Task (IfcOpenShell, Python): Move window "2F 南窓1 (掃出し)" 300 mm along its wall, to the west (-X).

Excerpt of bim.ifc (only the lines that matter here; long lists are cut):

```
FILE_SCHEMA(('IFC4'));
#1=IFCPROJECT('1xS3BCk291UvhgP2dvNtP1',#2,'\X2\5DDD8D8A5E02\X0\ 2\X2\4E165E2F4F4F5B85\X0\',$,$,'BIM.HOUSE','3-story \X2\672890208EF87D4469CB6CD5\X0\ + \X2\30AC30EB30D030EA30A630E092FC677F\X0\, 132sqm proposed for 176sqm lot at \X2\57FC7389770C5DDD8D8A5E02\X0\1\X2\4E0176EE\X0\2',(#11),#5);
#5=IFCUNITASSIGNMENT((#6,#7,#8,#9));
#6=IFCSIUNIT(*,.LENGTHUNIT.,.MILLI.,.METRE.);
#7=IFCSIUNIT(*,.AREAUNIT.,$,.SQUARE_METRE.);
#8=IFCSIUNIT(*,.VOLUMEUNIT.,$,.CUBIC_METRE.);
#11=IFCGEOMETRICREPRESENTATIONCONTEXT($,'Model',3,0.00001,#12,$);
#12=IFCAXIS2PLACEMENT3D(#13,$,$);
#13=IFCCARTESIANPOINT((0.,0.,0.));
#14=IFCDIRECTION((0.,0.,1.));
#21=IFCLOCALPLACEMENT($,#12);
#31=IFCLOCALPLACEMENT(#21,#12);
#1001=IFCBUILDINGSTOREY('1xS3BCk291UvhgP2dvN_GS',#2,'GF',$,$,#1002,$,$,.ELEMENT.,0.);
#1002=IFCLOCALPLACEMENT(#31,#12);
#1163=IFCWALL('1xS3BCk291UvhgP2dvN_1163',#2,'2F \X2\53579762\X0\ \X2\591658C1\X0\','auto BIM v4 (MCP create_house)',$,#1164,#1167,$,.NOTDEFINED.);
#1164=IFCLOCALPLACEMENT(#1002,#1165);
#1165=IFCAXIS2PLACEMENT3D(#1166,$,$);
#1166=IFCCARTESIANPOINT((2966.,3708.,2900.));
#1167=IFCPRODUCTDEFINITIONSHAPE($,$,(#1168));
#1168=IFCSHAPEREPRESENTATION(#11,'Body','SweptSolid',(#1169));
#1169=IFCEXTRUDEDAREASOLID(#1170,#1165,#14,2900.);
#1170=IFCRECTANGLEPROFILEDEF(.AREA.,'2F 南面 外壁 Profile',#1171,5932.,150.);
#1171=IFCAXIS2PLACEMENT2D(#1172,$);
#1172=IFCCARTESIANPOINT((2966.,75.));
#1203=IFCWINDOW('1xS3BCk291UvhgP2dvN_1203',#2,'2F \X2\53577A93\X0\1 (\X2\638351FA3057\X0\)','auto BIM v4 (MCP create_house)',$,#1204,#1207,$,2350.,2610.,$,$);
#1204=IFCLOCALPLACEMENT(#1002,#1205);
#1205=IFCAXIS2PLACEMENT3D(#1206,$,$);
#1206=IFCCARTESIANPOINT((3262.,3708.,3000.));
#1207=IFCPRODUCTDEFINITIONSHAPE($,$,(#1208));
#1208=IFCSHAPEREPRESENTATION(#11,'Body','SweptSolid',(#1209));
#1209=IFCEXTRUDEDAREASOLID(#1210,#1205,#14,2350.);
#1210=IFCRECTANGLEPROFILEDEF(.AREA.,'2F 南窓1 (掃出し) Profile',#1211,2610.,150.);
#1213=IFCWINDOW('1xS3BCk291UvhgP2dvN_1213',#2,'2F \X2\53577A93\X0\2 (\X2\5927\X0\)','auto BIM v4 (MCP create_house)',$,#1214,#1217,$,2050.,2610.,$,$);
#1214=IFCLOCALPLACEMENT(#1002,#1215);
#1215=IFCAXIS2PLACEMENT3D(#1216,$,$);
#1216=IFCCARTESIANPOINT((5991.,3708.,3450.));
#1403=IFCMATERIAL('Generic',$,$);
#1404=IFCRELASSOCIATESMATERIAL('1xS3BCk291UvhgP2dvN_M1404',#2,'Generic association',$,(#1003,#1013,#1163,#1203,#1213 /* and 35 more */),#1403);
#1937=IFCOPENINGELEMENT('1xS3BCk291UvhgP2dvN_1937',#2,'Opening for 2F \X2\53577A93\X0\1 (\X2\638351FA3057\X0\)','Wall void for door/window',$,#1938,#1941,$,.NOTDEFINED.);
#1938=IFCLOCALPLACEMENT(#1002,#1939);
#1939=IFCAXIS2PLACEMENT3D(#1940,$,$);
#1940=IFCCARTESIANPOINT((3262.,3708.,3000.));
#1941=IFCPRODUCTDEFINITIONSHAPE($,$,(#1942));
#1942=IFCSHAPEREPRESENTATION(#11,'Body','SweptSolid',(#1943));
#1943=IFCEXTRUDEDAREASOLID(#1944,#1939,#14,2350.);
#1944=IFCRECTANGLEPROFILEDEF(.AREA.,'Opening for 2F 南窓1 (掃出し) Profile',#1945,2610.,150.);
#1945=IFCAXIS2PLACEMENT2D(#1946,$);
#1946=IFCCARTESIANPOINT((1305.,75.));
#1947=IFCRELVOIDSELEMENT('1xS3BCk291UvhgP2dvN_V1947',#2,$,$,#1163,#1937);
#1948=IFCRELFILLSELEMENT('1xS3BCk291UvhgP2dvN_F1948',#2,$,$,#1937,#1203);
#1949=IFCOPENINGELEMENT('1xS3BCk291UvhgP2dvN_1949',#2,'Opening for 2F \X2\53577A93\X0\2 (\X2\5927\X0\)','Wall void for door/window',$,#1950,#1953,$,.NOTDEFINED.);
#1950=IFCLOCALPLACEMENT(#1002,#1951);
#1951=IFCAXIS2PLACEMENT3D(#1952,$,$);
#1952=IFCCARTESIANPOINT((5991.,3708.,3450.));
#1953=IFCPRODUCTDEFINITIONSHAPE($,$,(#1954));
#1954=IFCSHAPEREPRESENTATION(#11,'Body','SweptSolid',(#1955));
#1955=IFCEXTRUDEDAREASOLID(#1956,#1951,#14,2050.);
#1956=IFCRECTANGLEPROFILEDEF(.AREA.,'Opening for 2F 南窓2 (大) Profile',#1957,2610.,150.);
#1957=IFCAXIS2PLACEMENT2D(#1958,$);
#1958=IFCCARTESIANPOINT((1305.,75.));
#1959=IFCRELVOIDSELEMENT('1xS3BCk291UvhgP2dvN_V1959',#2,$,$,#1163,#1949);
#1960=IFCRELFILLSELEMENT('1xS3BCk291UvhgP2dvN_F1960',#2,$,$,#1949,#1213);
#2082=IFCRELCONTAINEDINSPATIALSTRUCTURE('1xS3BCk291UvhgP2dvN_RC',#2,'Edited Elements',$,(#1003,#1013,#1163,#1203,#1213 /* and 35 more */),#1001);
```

```python
import ifcopenshell
import ifcopenshell.api.geometry
import ifcopenshell.util.placement

model = ifcopenshell.open("bim.ifc")

window = model.by_id(1203)
opening = window.FillsVoids[0].RelatingOpeningElement
wall = opening.VoidsElements[0].RelatingBuildingElement

wall_matrix = ifcopenshell.util.placement.get_local_placement(wall.ObjectPlacement)
shift = wall_matrix[:3, 0] * -300.0
before = ifcopenshell.util.placement.get_local_placement(window.ObjectPlacement)[:3, 3].copy()

# The window is not placed relative to its opening, so move both.
for product in (opening, window):
    matrix = ifcopenshell.util.placement.get_local_placement(product.ObjectPlacement)
    matrix[:3, 3] += shift
    ifcopenshell.api.geometry.edit_object_placement(model, product=product, matrix=matrix, is_si=False)

after = ifcopenshell.util.placement.get_local_placement(window.ObjectPlacement)[:3, 3]
print("window moved by", (after - before).round(3) + 0.0)

model.write("bim_v2.ifc")
```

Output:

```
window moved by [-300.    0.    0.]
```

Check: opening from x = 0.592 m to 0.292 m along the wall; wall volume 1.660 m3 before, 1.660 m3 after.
